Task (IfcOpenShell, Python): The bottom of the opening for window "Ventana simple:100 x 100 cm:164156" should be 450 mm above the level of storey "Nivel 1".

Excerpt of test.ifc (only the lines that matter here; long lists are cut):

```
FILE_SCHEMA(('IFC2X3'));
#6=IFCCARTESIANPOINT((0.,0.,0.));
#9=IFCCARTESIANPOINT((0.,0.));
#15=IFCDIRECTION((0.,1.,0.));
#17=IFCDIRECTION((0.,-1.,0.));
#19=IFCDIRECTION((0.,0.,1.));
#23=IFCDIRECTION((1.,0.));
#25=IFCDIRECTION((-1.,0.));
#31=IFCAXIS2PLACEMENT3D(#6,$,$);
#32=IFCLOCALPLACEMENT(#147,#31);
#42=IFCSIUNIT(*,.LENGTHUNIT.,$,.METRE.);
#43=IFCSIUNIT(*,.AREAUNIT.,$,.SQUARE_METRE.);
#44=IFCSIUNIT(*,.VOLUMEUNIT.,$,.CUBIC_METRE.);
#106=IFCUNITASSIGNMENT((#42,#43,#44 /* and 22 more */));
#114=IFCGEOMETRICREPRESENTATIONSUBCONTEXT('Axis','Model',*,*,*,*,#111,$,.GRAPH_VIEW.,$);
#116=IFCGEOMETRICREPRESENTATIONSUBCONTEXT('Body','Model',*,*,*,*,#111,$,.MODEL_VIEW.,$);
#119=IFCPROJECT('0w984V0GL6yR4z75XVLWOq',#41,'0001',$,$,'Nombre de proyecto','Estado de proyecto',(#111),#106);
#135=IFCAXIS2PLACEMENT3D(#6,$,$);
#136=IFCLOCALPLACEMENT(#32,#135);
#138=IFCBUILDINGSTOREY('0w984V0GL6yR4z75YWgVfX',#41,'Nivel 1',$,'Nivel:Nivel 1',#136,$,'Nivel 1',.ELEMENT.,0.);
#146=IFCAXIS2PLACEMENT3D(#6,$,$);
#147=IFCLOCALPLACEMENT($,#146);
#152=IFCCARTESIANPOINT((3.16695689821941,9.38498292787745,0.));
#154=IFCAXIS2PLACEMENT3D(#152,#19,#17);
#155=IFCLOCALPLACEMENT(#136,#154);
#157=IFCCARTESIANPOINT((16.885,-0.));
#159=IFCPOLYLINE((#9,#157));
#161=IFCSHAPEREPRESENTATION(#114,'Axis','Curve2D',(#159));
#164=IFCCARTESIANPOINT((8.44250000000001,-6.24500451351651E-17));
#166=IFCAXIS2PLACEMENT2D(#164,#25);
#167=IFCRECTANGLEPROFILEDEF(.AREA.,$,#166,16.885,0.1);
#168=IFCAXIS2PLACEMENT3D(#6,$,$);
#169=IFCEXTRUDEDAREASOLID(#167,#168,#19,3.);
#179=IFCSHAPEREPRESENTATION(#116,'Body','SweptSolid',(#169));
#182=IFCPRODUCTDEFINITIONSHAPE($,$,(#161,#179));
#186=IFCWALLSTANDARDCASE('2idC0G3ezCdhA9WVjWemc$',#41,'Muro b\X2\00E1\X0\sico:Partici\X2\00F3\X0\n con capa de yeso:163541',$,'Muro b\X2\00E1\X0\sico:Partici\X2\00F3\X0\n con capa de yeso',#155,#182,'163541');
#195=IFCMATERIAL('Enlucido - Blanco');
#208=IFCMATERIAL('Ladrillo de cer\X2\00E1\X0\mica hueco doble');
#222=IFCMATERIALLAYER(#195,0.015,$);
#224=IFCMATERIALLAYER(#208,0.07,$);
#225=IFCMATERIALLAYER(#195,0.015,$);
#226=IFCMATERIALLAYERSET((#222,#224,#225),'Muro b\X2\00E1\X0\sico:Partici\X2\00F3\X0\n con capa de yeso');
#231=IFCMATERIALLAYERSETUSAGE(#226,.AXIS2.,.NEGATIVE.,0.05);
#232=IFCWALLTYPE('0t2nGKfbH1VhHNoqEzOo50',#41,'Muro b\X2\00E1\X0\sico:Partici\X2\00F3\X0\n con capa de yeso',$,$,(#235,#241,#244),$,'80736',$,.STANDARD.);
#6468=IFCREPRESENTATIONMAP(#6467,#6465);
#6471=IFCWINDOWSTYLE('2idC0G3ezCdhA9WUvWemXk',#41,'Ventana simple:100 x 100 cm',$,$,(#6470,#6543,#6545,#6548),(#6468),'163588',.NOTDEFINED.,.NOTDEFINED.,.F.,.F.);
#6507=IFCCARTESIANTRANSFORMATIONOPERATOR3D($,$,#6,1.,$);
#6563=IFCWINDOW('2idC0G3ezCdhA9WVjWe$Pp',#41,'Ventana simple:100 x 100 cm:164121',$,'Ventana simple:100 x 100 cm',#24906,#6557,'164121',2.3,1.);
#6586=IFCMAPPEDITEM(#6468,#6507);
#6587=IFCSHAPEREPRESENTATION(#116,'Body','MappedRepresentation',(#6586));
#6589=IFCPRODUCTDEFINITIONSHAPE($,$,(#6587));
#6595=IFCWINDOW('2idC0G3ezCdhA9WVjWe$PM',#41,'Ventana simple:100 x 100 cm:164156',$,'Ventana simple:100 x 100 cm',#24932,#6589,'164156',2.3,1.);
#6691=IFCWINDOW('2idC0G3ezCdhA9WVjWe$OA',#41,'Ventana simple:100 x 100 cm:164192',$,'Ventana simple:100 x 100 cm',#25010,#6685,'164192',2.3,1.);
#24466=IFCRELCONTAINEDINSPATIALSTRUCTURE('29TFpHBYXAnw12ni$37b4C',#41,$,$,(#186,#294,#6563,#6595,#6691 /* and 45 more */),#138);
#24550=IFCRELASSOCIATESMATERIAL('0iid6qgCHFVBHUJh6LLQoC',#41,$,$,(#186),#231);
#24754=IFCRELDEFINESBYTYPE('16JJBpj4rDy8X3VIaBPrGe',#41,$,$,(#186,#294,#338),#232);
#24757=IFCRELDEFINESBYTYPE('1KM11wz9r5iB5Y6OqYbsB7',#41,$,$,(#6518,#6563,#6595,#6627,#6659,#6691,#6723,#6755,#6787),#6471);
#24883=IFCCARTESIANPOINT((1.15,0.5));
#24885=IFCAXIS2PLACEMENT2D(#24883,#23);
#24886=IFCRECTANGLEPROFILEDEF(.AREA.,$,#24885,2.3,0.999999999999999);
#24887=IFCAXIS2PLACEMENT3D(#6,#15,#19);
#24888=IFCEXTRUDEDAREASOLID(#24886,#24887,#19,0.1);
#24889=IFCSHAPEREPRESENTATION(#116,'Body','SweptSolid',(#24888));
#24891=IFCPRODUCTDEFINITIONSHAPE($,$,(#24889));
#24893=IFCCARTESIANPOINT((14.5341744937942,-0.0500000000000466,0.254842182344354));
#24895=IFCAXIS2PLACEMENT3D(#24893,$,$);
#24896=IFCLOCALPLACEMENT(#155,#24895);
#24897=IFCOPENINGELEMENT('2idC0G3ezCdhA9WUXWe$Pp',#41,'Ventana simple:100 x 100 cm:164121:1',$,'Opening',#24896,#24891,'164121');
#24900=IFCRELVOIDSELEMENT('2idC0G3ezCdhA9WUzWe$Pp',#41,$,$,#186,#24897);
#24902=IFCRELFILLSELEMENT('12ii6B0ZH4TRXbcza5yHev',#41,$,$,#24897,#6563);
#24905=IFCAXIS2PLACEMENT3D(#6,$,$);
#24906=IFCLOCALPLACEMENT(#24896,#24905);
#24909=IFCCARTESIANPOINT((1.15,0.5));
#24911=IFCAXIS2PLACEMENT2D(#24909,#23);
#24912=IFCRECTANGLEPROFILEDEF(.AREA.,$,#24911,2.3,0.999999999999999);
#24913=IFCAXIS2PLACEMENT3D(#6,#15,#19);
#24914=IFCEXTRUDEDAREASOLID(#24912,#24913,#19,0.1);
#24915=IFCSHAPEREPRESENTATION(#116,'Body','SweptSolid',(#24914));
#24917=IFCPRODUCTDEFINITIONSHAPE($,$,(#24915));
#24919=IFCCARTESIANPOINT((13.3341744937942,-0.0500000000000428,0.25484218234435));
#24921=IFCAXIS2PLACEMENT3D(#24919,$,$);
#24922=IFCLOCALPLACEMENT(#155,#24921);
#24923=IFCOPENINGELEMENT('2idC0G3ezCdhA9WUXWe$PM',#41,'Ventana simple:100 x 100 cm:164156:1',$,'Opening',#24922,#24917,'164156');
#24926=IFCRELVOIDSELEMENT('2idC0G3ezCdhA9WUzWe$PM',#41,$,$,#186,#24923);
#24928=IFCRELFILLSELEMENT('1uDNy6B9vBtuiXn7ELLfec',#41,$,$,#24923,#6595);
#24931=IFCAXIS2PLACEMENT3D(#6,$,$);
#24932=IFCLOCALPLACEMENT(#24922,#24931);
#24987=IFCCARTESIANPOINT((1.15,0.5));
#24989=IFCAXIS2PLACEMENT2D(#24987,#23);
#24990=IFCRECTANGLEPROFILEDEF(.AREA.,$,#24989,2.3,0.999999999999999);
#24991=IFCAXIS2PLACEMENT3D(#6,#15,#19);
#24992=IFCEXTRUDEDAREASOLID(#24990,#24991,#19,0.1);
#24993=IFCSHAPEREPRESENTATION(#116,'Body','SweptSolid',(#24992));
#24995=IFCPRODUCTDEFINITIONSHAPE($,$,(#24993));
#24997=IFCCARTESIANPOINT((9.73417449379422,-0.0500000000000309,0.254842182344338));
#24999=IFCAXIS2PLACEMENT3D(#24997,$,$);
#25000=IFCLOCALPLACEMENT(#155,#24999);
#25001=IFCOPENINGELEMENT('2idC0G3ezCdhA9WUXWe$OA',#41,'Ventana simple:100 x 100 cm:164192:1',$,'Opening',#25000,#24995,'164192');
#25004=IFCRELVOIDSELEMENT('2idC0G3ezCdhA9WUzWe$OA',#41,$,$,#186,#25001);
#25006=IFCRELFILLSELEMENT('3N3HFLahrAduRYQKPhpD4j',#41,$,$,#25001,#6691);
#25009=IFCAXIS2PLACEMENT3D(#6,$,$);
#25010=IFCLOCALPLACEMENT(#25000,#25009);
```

```python
import numpy as np
import ifcopenshell
import ifcopenshell.api.geometry
import ifcopenshell.geom
import ifcopenshell.util.element
import ifcopenshell.util.placement
import ifcopenshell.util.shape
import ifcopenshell.util.unit

model = ifcopenshell.open("test.ifc")
unit_scale = ifcopenshell.util.unit.calculate_unit_scale(model)

window = model.by_guid("2idC0G3ezCdhA9WVjWe$PM")
opening = window.FillsVoids[0].RelatingOpeningElement
storey = ifcopenshell.util.element.get_container(window, ifc_class="IfcBuildingStorey")
level = ifcopenshell.util.placement.get_local_placement(storey.ObjectPlacement)[2, 3]

# The opening's origin need not be at the sill, so measure its lowest point.
shape = ifcopenshell.geom.create_shape(ifcopenshell.geom.settings(), opening)
bottom = ifcopenshell.util.shape.get_shape_bottom_elevation(shape, shape.geometry) / unit_scale
dz = level + 0.45 / unit_scale - bottom

shift = np.array([0.0, 0.0, dz])
# The window is placed relative to its opening, so it follows when the opening moves.
matrix = ifcopenshell.util.placement.get_local_placement(opening.ObjectPlacement)
matrix[:3, 3] += shift
ifcopenshell.api.geometry.edit_object_placement(
    model, product=opening, matrix=matrix, is_si=False, should_transform_children=True
)

print(f"moved by {dz * unit_scale:+.3f} m")

model.write("test-out.ifc")
```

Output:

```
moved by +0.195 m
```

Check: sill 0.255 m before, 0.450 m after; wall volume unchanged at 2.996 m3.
